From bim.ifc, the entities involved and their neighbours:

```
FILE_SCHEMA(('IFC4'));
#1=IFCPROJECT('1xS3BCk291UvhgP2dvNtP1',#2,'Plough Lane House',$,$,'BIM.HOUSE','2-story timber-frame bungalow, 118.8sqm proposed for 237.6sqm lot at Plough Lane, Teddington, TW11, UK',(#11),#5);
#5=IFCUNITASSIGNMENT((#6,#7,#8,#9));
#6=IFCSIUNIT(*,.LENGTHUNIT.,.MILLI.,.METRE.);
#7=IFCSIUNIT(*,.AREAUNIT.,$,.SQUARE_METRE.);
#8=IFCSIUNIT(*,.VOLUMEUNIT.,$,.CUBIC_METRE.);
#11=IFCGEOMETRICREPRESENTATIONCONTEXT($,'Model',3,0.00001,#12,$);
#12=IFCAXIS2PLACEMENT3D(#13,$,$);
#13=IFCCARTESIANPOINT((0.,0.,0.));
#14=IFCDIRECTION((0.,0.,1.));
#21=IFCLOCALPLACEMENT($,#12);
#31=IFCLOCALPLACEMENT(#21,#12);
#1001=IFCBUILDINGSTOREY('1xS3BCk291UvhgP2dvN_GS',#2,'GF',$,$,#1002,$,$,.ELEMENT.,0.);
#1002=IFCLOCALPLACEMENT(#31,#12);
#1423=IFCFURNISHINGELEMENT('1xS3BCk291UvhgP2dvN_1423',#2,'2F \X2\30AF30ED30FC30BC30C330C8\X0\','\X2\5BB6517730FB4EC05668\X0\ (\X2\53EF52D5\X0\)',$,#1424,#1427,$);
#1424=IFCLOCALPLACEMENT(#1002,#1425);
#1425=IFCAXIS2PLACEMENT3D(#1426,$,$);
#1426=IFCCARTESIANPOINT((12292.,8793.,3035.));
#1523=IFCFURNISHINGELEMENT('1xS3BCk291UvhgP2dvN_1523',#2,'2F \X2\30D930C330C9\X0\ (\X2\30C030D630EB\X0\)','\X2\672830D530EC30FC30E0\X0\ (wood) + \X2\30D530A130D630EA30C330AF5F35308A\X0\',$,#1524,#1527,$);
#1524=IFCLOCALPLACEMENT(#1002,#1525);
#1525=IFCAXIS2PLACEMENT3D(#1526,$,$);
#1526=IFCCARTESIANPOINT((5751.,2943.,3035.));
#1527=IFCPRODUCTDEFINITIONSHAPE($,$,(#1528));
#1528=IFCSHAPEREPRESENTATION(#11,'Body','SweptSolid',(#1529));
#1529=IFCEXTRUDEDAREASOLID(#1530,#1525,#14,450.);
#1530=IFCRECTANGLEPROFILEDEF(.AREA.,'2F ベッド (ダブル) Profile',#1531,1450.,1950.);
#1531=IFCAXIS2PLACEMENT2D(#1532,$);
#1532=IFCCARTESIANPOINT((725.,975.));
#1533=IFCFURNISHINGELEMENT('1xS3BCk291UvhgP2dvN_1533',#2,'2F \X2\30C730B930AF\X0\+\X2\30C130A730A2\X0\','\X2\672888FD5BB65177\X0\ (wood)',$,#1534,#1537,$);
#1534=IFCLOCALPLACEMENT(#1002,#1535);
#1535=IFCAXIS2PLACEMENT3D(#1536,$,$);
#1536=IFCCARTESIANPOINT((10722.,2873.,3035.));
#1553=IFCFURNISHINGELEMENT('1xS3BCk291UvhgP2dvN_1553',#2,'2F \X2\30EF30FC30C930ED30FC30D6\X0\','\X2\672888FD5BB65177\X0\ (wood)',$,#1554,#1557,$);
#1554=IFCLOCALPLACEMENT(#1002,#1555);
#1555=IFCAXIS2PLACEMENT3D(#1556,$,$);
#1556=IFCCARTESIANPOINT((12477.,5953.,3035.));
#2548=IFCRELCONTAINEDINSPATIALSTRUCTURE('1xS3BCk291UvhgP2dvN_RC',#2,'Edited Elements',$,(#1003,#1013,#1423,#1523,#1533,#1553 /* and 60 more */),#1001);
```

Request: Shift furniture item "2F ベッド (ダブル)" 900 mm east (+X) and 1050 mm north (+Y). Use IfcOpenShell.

```python
import ifcopenshell
import ifcopenshell.api.geometry
import ifcopenshell.util.placement
import ifcopenshell.util.unit

model = ifcopenshell.open("bim.ifc")
unit_scale = ifcopenshell.util.unit.calculate_unit_scale(model)

item = model.by_id(1523)
matrix = ifcopenshell.util.placement.get_local_placement(item.ObjectPlacement)
matrix[0, 3] += 0.9 / unit_scale
matrix[1, 3] += 1.05 / unit_scale
ifcopenshell.api.geometry.edit_object_placement(model, product=item, matrix=matrix, is_si=False)

print(ifcopenshell.util.placement.get_local_placement(item.ObjectPlacement).round(3) + 0.0)

model.write("bim_v2.ifc")
```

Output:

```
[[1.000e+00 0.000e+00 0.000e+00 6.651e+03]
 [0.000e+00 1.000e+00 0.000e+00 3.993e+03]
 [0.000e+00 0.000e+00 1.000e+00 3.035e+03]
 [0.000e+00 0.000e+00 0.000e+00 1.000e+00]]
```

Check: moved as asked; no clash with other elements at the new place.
